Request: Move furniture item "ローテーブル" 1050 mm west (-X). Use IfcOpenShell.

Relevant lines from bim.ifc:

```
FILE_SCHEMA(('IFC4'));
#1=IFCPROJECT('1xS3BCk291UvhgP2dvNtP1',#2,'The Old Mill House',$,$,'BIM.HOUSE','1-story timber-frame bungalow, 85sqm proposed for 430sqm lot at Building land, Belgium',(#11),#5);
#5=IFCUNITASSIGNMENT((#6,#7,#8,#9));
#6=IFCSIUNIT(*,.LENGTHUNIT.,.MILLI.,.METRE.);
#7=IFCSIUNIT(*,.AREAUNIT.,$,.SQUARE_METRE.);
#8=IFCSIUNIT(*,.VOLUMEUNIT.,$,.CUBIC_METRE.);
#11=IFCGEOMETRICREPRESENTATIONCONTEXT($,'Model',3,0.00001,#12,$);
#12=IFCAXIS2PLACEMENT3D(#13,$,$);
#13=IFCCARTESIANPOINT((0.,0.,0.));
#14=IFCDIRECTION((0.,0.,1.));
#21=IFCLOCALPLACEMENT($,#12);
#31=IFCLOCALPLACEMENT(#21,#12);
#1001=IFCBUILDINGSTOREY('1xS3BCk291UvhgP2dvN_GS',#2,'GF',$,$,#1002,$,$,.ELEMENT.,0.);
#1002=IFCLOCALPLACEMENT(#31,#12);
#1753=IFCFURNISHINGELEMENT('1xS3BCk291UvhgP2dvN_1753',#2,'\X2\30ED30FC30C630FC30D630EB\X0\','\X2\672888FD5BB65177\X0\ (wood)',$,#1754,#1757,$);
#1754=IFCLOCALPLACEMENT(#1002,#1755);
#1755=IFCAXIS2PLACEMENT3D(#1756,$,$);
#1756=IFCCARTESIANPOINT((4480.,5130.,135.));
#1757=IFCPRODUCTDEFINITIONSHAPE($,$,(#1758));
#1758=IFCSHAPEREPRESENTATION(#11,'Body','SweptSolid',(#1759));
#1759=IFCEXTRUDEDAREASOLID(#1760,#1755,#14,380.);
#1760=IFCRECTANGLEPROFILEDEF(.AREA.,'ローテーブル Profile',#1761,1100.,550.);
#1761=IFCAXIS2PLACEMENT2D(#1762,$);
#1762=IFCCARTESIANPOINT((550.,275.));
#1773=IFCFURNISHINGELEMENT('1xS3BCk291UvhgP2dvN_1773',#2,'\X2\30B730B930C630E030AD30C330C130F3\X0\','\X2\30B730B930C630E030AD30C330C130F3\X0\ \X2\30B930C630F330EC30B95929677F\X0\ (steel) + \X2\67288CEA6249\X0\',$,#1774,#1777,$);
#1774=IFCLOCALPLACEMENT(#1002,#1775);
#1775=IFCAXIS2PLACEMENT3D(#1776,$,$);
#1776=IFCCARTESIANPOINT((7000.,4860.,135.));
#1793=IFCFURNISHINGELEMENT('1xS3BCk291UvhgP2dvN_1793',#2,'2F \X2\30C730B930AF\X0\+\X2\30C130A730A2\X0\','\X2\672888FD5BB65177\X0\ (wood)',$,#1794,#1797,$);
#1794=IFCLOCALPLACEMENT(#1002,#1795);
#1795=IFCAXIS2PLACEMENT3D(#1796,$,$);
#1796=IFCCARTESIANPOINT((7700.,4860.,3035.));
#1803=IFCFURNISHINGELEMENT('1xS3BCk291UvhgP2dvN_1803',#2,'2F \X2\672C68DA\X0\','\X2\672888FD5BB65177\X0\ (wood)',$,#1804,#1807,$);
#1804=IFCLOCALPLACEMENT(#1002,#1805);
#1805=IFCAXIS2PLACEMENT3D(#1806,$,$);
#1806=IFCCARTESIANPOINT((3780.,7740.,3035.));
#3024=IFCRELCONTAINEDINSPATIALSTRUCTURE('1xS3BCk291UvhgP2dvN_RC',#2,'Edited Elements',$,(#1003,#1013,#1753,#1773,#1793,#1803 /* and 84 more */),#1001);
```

```python
import ifcopenshell
import ifcopenshell.api.geometry
import ifcopenshell.util.placement

model = ifcopenshell.open("bim.ifc")

item = model.by_guid("1xS3BCk291UvhgP2dvN_1753")
matrix = ifcopenshell.util.placement.get_local_placement(item.ObjectPlacement)
matrix[0, 3] -= 1050.0
ifcopenshell.api.geometry.edit_object_placement(model, product=item, matrix=matrix, is_si=False)

print(ifcopenshell.util.placement.get_local_placement(item.ObjectPlacement).round(3) + 0.0)

model.write("bim_edited.ifc")
```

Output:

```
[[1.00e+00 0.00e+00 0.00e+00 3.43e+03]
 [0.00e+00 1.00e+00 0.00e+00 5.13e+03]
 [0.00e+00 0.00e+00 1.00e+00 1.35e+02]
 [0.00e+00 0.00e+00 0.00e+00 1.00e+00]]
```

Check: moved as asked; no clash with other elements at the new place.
